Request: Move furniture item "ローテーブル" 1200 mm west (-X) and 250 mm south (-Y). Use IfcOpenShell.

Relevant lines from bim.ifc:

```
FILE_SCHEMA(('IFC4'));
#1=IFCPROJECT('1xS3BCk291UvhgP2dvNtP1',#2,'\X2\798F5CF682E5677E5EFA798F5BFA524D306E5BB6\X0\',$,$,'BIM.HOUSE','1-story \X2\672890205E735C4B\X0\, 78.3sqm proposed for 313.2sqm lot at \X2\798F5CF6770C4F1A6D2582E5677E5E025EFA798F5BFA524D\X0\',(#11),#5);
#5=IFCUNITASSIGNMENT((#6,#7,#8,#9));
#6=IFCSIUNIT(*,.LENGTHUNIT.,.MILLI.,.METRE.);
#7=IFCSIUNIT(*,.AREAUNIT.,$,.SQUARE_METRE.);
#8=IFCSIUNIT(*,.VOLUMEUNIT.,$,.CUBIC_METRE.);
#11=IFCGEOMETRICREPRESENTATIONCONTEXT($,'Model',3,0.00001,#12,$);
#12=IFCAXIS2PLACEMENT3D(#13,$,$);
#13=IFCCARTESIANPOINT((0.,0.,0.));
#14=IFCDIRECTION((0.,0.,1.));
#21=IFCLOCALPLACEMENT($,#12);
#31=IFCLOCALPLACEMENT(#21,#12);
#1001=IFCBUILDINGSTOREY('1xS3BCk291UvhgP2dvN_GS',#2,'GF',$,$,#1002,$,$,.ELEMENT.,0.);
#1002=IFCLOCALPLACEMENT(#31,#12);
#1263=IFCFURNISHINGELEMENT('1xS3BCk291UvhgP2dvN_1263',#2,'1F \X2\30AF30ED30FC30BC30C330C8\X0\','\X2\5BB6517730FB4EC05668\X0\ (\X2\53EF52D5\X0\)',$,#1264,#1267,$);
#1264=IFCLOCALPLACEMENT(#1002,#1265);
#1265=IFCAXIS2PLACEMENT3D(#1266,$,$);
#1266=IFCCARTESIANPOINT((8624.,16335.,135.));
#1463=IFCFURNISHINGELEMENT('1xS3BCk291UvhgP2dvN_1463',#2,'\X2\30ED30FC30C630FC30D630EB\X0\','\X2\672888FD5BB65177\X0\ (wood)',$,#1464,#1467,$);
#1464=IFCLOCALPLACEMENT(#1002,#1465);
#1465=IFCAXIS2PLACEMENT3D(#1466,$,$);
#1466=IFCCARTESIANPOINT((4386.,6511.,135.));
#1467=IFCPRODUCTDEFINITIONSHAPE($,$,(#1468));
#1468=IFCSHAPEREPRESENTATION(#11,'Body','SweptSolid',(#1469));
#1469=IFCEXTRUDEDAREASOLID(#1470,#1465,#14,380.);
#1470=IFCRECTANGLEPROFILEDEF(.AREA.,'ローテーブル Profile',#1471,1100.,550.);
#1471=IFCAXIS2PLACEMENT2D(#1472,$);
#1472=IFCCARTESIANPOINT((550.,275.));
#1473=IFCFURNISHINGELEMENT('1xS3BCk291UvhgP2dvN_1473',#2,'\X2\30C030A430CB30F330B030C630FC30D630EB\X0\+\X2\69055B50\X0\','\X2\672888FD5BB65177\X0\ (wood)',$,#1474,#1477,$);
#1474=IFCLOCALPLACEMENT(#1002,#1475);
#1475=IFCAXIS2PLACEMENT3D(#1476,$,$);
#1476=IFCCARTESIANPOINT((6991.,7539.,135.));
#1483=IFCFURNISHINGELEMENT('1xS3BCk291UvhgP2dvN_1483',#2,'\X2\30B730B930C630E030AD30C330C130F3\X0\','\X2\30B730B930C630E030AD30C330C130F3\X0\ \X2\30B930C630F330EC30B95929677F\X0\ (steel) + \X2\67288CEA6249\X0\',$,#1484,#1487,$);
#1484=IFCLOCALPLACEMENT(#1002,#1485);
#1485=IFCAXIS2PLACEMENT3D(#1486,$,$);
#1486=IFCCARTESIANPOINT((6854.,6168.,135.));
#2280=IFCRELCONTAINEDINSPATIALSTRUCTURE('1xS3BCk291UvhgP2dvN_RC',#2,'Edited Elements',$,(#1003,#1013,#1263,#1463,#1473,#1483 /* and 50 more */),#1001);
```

```python
import ifcopenshell
import ifcopenshell.api.geometry
import ifcopenshell.util.placement
import ifcopenshell.util.unit

model = ifcopenshell.open("bim.ifc")
unit_scale = ifcopenshell.util.unit.calculate_unit_scale(model)

item = model.by_guid("1xS3BCk291UvhgP2dvN_1463")
matrix = ifcopenshell.util.placement.get_local_placement(item.ObjectPlacement)
matrix[0, 3] -= 1.2 / unit_scale
matrix[1, 3] -= 0.25 / unit_scale
ifcopenshell.api.geometry.edit_object_placement(model, product=item, matrix=matrix, is_si=False)

print(ifcopenshell.util.placement.get_local_placement(item.ObjectPlacement).round(3) + 0.0)

model.write("bim-out.ifc")
```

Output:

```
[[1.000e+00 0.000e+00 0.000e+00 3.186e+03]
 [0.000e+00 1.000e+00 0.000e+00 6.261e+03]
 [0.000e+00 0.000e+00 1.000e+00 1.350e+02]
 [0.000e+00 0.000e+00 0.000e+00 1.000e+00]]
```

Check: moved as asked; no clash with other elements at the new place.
